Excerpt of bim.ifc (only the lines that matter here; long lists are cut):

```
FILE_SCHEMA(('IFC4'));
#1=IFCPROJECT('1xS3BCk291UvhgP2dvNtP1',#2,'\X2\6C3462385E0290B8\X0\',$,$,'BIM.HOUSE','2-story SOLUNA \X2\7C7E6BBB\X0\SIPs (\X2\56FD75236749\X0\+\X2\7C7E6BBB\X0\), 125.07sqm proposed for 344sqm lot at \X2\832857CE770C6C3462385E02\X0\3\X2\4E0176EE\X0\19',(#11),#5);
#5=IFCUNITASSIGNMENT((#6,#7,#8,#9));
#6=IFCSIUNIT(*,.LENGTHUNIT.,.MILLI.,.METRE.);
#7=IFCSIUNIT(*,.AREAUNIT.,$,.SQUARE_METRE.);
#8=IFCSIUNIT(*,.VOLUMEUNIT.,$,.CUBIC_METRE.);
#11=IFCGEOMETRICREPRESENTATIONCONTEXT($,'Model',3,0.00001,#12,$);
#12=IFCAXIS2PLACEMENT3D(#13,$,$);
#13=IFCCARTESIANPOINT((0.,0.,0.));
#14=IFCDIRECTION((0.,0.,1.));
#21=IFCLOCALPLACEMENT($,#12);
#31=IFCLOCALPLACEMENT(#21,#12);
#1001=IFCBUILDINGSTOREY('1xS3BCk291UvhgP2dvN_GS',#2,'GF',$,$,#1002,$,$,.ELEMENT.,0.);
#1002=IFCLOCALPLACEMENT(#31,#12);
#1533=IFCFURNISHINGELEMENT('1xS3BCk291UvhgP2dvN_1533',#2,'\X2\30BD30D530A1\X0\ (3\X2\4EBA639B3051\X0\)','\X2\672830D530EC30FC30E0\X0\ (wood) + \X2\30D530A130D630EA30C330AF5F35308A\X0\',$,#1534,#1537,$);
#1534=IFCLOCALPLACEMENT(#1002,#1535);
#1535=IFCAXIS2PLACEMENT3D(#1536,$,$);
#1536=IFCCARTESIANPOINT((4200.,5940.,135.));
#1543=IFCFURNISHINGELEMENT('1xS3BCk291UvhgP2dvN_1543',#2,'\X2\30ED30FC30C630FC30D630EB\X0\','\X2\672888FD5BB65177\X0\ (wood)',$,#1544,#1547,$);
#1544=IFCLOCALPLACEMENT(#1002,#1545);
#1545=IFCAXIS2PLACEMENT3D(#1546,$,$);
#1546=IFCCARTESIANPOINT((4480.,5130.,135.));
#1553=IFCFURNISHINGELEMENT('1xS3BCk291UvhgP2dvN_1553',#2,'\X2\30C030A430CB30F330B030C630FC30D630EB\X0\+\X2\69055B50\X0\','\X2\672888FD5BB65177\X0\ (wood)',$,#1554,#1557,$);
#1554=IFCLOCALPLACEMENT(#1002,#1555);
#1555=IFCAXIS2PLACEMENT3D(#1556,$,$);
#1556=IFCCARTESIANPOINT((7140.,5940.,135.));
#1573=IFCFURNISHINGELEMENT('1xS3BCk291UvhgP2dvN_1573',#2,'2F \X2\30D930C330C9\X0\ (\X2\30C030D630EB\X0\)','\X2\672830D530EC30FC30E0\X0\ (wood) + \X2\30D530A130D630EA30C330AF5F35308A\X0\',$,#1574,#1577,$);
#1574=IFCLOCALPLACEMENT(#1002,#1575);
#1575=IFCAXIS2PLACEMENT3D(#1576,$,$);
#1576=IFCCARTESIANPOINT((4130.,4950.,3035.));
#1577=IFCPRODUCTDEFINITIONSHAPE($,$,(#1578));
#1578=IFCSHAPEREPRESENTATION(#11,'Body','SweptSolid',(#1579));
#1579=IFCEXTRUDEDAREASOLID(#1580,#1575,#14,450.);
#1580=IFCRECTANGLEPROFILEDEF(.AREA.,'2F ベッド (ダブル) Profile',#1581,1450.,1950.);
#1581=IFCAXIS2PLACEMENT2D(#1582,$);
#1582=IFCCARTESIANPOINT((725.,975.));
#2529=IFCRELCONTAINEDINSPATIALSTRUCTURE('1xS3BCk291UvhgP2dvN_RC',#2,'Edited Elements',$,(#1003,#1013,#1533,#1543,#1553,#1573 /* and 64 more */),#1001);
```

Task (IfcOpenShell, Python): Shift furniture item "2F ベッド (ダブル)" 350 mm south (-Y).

```python
import ifcopenshell
import ifcopenshell.api.geometry
import ifcopenshell.util.placement

model = ifcopenshell.open("bim.ifc")

item = model.by_guid("1xS3BCk291UvhgP2dvN_1573")
matrix = ifcopenshell.util.placement.get_local_placement(item.ObjectPlacement)
matrix[1, 3] -= 350.0
ifcopenshell.api.geometry.edit_object_placement(model, product=item, matrix=matrix, is_si=False)

print(ifcopenshell.util.placement.get_local_placement(item.ObjectPlacement).round(3) + 0.0)

model.write("bim_edited.ifc")
```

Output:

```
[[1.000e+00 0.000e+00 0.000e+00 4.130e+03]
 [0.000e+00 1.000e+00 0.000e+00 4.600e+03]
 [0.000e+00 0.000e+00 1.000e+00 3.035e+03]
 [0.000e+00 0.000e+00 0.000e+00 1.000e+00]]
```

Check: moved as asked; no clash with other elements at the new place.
